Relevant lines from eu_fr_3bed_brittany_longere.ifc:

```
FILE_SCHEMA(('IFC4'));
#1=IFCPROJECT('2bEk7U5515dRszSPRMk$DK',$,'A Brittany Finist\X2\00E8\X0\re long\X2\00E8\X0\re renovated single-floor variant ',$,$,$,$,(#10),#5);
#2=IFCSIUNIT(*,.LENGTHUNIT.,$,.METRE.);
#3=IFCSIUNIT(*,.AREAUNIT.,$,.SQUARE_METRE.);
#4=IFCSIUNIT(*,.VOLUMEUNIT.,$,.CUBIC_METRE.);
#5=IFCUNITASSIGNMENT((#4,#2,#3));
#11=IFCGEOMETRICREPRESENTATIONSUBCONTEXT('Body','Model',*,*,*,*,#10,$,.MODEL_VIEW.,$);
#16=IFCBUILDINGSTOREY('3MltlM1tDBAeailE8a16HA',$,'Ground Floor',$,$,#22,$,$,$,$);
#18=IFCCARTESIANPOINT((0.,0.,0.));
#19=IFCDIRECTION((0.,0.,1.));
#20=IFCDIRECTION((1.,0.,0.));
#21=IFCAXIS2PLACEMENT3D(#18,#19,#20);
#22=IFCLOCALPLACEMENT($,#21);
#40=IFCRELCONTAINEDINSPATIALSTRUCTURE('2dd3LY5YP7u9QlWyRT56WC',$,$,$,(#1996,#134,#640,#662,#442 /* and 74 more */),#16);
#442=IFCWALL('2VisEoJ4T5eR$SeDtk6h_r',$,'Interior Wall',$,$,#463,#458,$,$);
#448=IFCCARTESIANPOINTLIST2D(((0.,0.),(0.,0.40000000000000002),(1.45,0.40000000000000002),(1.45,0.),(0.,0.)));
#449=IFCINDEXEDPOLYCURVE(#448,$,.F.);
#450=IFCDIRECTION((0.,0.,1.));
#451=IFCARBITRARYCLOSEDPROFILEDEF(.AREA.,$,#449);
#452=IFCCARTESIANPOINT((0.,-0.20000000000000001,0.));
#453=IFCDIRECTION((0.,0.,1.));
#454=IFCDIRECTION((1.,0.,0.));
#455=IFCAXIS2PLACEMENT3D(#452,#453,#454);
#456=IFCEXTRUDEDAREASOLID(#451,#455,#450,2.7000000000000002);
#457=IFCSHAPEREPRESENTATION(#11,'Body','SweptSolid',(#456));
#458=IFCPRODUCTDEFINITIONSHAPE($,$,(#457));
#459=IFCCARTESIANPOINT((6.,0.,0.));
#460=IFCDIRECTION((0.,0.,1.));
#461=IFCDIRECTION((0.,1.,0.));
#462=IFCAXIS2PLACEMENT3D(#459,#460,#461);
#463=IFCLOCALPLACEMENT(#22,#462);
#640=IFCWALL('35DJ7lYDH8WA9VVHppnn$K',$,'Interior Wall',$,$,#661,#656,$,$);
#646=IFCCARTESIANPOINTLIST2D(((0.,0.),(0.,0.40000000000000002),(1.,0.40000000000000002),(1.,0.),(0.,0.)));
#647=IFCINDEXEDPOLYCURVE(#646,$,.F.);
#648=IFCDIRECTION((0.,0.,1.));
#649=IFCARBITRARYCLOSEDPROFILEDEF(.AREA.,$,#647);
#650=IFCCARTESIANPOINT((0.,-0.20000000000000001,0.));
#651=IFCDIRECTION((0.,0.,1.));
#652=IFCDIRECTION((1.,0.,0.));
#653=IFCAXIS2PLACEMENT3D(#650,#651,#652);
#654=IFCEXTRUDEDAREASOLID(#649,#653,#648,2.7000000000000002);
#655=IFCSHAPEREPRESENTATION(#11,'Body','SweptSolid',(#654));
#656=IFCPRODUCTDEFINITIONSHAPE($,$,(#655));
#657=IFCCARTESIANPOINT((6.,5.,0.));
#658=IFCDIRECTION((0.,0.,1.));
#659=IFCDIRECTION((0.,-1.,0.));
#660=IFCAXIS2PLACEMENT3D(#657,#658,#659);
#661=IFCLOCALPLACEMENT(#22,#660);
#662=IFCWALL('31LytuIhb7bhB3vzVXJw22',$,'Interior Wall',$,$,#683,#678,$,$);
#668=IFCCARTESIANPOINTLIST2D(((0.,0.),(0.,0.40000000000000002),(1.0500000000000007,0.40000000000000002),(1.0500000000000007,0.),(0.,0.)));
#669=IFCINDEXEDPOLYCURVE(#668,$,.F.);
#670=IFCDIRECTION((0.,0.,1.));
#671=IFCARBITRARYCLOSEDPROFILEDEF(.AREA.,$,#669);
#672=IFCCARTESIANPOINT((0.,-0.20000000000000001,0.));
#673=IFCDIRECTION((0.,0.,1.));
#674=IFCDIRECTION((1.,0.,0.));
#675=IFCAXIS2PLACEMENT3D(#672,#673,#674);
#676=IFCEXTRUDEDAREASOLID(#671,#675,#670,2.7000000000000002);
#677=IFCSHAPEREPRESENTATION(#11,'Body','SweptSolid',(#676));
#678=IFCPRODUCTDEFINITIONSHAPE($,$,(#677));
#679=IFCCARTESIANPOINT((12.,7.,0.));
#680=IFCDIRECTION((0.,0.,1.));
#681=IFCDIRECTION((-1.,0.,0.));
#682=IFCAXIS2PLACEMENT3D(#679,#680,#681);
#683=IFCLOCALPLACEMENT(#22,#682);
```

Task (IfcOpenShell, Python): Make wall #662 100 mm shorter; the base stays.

```python
import ifcopenshell
import ifcopenshell.geom
import ifcopenshell.util.representation
import ifcopenshell.util.shape
import ifcopenshell.util.unit

model = ifcopenshell.open("eu_fr_3bed_brittany_longere.ifc")
unit_scale = ifcopenshell.util.unit.calculate_unit_scale(model)
settings = ifcopenshell.geom.settings()


def volume(element):
    """Net volume in cubic metres, openings subtracted."""
    shape = ifcopenshell.geom.create_shape(settings, element)
    return ifcopenshell.util.shape.get_volume(shape.geometry)


wall = model.by_id(662)
before = volume(wall)

body = ifcopenshell.util.representation.get_representation(wall, "Model", "Body")
solid = body.Items[0]
old_height = solid.Depth
solid.Depth -= 0.1 / unit_scale
after = volume(wall)

print(f"height {old_height:g} -> {solid.Depth:g}, volume {before:.3f} -> {after:.3f} m3")

model.write("eu_fr_3bed_brittany_longere_rev.ifc")
```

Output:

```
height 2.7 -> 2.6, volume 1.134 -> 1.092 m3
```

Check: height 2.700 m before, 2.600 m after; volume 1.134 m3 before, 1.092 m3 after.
